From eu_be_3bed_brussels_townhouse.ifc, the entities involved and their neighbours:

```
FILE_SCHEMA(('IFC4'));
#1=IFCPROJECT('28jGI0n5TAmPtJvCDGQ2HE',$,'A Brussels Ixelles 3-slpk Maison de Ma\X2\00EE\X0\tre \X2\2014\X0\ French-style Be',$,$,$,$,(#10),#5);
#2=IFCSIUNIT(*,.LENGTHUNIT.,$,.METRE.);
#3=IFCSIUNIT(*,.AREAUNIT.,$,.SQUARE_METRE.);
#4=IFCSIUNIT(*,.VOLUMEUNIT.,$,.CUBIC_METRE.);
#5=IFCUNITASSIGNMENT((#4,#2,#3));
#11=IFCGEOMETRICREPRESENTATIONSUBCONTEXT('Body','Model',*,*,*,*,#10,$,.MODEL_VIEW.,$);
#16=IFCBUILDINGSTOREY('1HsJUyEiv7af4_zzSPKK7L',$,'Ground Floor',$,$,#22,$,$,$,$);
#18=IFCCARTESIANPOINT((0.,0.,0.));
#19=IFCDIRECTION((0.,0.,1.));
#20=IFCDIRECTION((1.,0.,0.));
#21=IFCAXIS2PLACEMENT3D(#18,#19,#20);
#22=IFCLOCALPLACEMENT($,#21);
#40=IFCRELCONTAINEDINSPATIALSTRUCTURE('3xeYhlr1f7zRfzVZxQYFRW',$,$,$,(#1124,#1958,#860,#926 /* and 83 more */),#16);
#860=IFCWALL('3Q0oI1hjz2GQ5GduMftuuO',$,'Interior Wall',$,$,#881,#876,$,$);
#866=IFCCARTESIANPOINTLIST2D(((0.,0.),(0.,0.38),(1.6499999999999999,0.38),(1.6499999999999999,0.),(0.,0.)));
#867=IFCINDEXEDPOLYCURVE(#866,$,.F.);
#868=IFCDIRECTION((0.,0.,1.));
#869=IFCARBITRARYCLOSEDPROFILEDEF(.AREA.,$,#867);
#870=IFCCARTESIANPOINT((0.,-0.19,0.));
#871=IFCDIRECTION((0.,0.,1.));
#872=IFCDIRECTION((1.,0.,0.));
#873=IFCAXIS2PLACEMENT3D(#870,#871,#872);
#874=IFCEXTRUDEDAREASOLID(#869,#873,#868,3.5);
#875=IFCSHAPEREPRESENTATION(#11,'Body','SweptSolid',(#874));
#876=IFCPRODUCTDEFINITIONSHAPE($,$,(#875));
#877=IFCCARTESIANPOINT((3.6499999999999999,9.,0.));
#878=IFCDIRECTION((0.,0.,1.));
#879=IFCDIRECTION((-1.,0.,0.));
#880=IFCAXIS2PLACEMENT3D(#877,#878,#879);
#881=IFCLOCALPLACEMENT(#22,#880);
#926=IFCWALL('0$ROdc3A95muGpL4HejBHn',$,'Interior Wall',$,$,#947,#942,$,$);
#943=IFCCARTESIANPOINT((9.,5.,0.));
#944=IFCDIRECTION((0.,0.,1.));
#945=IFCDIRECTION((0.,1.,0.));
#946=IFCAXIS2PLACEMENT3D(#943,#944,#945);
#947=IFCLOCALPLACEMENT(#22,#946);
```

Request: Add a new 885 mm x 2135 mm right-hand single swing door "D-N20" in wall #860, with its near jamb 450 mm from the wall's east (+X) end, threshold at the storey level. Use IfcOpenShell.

```python
import numpy as np
import ifcopenshell
import ifcopenshell.api.feature
import ifcopenshell.api.geometry
import ifcopenshell.api.root
import ifcopenshell.api.spatial
import ifcopenshell.geom
import ifcopenshell.util.element
import ifcopenshell.util.placement
import ifcopenshell.util.representation
import ifcopenshell.util.shape
import ifcopenshell.util.unit

model = ifcopenshell.open("eu_be_3bed_brussels_townhouse.ifc")
unit_scale = ifcopenshell.util.unit.calculate_unit_scale(model)
settings = ifcopenshell.geom.settings()


def volume(element):
    """Net volume in cubic metres, openings subtracted."""
    shape = ifcopenshell.geom.create_shape(settings, element)
    return ifcopenshell.util.shape.get_volume(shape.geometry)


wall = model.by_guid("3Q0oI1hjz2GQ5GduMftuuO")
storey = ifcopenshell.util.element.get_container(wall, ifc_class="IfcBuildingStorey")
context = ifcopenshell.util.representation.get_context(model, "Model", "Body", "MODEL_VIEW")
before = volume(wall)

width, height, from_end, sill = 0.885, 2.135, 0.45, 0.0  # metres

# The wall runs along its own X axis, and the end named is its -X end.
wall_shape = ifcopenshell.geom.create_shape(settings, wall)
x, y, z = ifcopenshell.util.shape.get_vertices(wall_shape.geometry).T
start = x.min() + from_end
face, thickness = float(y.min()), float(y.max() - y.min())
wall_matrix = ifcopenshell.util.placement.get_local_placement(wall.ObjectPlacement)
level = ifcopenshell.util.placement.get_local_placement(storey.ObjectPlacement)[2, 3]


def in_wall(x, y):
    """Placement at x, y metres in the wall's axes, at sill height."""
    matrix = wall_matrix.copy()
    matrix[:, 3] = wall_matrix @ np.array([x / unit_scale, y / unit_scale, 0.0, 1.0])
    matrix[2, 3] = level + sill / unit_scale
    return matrix


# Opening: a box that overshoots both wall faces by 50 mm.
opening = ifcopenshell.api.root.create_entity(model, ifc_class="IfcOpeningElement", predefined_type="OPENING")
box = ifcopenshell.api.geometry.add_wall_representation(
    model, context=context, length=width, height=height, thickness=thickness + 0.1
)
ifcopenshell.api.geometry.assign_representation(model, product=opening, representation=box)
ifcopenshell.api.geometry.edit_object_placement(model, product=opening, matrix=in_wall(start, face - 0.05), is_si=False)
ifcopenshell.api.feature.add_feature(model, feature=opening, element=wall)

door = ifcopenshell.api.root.create_entity(model, ifc_class="IfcDoor", name="D-N20", predefined_type="DOOR")
door.OverallWidth, door.OverallHeight = width / unit_scale, height / unit_scale
door.OperationType = "SINGLE_SWING_RIGHT"
body = ifcopenshell.api.geometry.add_door_representation(
    model,
    context=context,
    overall_width=door.OverallWidth,
    overall_height=door.OverallHeight,
    operation_type="SINGLE_SWING_RIGHT",
    lining_properties={"LiningDepth": thickness / unit_scale, "ThresholdDepth": thickness / unit_scale},
)
ifcopenshell.api.geometry.assign_representation(model, product=door, representation=body)
ifcopenshell.api.spatial.assign_container(model, products=[door], relating_structure=storey)
ifcopenshell.api.feature.add_filling(model, opening=opening, element=door)

# The lining spans the wall, so the door starts at the wall face.
ifcopenshell.api.geometry.edit_object_placement(model, product=door, matrix=in_wall(start, face), is_si=False)

after = volume(wall)

print(f"wall volume {before:.3f} -> {after:.3f} m3")

model.write("eu_be_3bed_brussels_townhouse_v2.ifc")
```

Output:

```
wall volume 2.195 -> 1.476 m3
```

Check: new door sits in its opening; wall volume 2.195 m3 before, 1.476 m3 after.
